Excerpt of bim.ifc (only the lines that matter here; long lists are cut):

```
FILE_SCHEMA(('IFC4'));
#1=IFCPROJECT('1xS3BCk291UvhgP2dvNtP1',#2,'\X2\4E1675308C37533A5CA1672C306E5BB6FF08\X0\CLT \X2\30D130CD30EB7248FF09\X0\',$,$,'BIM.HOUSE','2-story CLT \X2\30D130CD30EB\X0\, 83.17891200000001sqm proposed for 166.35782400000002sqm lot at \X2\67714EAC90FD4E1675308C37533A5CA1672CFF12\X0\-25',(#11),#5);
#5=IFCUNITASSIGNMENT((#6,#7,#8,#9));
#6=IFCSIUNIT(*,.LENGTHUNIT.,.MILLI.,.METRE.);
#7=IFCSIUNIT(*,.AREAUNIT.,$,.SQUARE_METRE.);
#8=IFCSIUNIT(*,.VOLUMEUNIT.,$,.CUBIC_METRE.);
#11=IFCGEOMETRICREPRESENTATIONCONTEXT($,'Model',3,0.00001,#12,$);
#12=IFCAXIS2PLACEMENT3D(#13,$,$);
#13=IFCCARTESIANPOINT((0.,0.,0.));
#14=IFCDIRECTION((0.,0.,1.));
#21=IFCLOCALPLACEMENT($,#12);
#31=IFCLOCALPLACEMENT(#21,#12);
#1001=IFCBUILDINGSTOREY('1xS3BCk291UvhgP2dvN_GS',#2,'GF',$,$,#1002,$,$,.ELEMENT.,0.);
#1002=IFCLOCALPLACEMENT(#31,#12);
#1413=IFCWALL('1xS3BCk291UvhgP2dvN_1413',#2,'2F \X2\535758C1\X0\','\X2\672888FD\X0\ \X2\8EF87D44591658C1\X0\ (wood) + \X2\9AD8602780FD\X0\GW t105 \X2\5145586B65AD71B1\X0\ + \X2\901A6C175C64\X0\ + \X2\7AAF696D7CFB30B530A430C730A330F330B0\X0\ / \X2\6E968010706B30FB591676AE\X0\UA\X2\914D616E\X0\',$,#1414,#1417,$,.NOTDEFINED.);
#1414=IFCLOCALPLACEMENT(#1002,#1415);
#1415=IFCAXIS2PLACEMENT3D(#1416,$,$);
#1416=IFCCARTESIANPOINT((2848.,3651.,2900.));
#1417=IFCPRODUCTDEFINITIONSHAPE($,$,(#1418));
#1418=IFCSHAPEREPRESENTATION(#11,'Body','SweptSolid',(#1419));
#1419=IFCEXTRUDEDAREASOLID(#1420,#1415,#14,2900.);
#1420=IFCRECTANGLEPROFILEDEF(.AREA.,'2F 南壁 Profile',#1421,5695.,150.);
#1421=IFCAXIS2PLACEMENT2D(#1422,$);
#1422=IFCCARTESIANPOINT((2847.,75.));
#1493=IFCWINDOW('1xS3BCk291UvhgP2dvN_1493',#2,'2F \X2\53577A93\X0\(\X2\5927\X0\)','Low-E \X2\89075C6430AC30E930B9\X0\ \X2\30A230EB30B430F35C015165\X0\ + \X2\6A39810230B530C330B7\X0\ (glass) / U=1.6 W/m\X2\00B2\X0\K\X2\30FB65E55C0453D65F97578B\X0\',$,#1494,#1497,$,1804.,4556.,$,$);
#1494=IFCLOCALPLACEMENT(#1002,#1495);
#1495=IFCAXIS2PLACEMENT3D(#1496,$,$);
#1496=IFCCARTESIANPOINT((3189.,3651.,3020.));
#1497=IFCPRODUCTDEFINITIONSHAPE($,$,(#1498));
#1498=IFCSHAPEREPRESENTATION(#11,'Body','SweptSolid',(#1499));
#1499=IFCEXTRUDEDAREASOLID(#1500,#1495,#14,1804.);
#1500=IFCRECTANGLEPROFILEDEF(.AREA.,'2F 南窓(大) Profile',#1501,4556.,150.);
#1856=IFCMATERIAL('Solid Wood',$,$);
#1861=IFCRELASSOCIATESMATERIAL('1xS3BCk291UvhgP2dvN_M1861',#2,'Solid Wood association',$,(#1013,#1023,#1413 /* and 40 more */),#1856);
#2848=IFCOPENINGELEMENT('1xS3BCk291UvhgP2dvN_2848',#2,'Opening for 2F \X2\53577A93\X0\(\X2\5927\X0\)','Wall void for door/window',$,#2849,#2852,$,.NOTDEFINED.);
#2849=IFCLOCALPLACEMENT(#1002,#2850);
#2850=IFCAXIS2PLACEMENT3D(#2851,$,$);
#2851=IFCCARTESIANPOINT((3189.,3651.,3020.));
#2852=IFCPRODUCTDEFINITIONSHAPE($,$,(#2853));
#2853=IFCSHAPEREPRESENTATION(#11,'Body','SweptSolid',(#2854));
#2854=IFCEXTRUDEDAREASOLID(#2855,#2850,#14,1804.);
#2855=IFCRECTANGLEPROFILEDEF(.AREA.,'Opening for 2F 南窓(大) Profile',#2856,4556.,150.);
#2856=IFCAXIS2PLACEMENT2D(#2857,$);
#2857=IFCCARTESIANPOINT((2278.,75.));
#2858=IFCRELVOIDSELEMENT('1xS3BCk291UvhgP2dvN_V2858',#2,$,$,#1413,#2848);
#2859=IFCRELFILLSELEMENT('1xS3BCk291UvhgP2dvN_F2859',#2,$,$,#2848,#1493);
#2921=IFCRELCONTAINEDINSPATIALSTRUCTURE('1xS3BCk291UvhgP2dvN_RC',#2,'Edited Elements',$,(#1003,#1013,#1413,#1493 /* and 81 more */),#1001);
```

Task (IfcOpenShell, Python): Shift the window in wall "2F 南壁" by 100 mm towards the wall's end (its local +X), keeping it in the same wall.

```python
import ifcopenshell
import ifcopenshell.api.geometry
import ifcopenshell.util.placement
import ifcopenshell.util.unit

model = ifcopenshell.open("bim.ifc")
unit_scale = ifcopenshell.util.unit.calculate_unit_scale(model)

window = model.by_guid("1xS3BCk291UvhgP2dvN_1493")
opening = window.FillsVoids[0].RelatingOpeningElement
wall = opening.VoidsElements[0].RelatingBuildingElement

wall_matrix = ifcopenshell.util.placement.get_local_placement(wall.ObjectPlacement)
shift = wall_matrix[:3, 0] * 0.1 / unit_scale
before = ifcopenshell.util.placement.get_local_placement(window.ObjectPlacement)[:3, 3].copy()

# The window is not placed relative to its opening, so move both.
for product in (opening, window):
    matrix = ifcopenshell.util.placement.get_local_placement(product.ObjectPlacement)
    matrix[:3, 3] += shift
    ifcopenshell.api.geometry.edit_object_placement(model, product=product, matrix=matrix, is_si=False)

after = ifcopenshell.util.placement.get_local_placement(window.ObjectPlacement)[:3, 3]
print("window moved by", (after - before).round(3) + 0.0)

model.write("bim_v2.ifc")
```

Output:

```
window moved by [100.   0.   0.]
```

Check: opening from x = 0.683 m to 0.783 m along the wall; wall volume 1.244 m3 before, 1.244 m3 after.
